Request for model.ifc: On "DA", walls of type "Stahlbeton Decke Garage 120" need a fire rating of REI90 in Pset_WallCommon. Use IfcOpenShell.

First a look at what the model holds.

```python
import ifcopenshell
import ifcopenshell.util.element

model = ifcopenshell.open("model.ifc")
print(model.schema)
storey = next(s for s in model.by_type("IfcBuildingStorey") if s.Name == "DA")
walls = [e for e in ifcopenshell.util.element.get_decomposition(storey) if e.is_a("IfcWall")]
seen = {}
for e in walls:
    element_type = ifcopenshell.util.element.get_type(e)
    key = (element_type.Name if element_type != e and element_type else None, ifcopenshell.util.element.get_pset(e, "Pset_WallCommon", "FireRating"))
    seen[key] = seen.get(key, 0) + 1
for (name, value), count in sorted(seen.items(), key=str):
    print(count, "x", name, "|", value)
```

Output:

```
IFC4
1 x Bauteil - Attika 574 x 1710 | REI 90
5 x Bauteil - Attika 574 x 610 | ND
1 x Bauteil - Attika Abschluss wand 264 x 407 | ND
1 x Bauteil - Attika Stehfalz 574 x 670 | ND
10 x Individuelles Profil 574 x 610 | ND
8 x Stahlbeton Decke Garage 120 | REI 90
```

```python
import ifcopenshell
import ifcopenshell.api.pset
import ifcopenshell.util.element

model = ifcopenshell.open("model.ifc")

storey = next(s for s in model.by_type("IfcBuildingStorey") if s.Name == "DA")
walls = [e for e in ifcopenshell.util.element.get_decomposition(storey) if e.is_a("IfcWall")]

count = 0
for e in walls:
    element_type = ifcopenshell.util.element.get_type(e)
    if element_type in (None, e) or element_type.Name != "Stahlbeton Decke Garage 120":
        continue
    # add_pset returns the element's existing set when there is one.
    pset = ifcopenshell.api.pset.add_pset(model, product=e, name="Pset_WallCommon")
    ifcopenshell.api.pset.edit_pset(model, pset=pset, properties={"FireRating": "REI90"})
    count += 1

print(count, "walls updated")

model.write("model_rev.ifc")
```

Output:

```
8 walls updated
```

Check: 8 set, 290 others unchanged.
